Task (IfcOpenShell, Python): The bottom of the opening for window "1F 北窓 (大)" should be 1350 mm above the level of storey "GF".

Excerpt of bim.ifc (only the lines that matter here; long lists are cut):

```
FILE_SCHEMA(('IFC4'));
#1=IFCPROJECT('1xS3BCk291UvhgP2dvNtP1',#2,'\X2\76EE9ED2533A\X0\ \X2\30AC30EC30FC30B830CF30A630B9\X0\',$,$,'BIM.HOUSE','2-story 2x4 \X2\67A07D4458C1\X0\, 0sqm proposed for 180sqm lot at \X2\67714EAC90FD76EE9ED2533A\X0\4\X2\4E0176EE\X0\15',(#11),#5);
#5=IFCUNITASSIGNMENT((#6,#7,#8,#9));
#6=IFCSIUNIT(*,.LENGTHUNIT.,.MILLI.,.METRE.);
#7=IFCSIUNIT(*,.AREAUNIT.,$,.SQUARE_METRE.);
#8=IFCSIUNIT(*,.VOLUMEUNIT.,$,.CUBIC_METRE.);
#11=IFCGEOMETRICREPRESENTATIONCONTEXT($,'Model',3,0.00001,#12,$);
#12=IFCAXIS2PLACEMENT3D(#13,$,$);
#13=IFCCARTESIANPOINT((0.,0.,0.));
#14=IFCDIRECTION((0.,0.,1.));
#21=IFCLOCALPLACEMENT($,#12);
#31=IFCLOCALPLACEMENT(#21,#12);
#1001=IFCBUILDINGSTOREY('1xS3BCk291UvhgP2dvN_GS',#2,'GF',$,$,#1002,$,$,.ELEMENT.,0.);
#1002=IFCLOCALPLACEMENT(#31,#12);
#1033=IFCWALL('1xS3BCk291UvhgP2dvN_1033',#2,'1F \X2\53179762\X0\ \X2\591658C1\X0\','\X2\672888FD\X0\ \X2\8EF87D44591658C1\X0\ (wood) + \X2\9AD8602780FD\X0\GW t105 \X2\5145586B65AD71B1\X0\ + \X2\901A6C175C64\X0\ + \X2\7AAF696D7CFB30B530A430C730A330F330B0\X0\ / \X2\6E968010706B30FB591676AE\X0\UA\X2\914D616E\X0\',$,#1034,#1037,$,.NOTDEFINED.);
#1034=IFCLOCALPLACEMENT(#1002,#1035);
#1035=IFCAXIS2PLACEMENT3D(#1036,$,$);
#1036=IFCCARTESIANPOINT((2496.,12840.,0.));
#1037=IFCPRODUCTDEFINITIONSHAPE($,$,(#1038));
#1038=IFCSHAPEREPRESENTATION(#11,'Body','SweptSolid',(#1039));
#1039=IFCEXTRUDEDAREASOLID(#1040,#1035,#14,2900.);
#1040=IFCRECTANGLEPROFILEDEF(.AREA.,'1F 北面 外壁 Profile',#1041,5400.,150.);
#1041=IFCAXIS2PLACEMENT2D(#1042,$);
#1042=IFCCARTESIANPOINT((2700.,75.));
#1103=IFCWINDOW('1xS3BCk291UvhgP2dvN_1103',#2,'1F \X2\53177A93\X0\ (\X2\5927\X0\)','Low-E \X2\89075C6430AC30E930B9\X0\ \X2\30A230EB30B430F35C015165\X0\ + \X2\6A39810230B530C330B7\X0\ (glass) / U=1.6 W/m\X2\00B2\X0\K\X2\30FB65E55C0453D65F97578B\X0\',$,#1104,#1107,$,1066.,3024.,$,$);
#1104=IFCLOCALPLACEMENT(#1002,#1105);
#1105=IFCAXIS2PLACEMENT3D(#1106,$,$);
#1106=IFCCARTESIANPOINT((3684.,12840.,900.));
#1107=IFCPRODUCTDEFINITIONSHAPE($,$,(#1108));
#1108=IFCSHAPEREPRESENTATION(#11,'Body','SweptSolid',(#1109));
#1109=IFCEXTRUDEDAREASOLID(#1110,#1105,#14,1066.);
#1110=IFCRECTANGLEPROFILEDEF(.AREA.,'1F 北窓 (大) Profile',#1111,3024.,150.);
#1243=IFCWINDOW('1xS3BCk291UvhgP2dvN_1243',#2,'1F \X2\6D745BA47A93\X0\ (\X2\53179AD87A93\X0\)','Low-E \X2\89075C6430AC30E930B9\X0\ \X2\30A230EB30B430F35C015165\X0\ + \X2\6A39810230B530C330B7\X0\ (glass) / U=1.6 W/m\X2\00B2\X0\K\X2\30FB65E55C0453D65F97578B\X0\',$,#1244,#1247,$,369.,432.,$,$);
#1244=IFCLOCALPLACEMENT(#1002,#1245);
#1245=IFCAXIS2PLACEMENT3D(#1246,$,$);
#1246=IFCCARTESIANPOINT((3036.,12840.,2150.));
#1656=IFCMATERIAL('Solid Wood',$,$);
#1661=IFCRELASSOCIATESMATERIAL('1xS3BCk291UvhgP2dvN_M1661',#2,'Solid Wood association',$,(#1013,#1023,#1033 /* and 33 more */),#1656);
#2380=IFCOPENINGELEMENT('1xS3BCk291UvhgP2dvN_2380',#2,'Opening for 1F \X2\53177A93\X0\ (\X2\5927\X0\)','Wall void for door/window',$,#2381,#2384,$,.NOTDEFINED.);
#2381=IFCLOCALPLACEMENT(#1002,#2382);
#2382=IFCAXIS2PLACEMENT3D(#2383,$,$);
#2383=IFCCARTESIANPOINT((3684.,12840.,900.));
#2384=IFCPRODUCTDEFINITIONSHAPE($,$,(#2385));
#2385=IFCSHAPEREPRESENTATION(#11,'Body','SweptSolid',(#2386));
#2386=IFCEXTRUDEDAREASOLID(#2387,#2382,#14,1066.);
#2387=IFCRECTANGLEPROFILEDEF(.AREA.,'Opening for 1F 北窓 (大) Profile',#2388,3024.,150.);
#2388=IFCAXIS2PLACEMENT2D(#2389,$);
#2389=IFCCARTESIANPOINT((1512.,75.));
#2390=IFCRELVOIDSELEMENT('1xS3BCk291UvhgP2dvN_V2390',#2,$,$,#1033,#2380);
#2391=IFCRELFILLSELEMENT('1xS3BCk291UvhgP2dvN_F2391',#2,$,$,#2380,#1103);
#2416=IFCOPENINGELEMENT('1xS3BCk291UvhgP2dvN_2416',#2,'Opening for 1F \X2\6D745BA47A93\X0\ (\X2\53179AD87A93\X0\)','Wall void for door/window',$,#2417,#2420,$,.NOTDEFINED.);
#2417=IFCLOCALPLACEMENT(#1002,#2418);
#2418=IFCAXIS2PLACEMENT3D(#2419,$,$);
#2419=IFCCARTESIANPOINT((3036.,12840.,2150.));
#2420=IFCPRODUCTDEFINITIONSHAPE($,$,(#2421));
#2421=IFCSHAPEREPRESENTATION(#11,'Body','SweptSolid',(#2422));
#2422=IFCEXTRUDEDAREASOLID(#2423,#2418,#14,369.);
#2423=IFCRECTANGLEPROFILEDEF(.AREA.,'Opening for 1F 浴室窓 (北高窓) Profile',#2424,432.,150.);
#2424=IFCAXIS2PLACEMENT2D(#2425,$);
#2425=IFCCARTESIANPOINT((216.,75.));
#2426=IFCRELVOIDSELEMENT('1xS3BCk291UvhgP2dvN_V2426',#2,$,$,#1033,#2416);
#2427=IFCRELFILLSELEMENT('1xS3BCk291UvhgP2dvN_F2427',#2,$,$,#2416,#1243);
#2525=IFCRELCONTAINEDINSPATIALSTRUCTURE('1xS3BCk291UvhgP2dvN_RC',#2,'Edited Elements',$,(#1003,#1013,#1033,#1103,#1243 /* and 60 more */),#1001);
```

```python
import numpy as np
import ifcopenshell
import ifcopenshell.api.geometry
import ifcopenshell.geom
import ifcopenshell.util.element
import ifcopenshell.util.placement
import ifcopenshell.util.shape
import ifcopenshell.util.unit

model = ifcopenshell.open("bim.ifc")
unit_scale = ifcopenshell.util.unit.calculate_unit_scale(model)

window = model.by_guid("1xS3BCk291UvhgP2dvN_1103")
opening = window.FillsVoids[0].RelatingOpeningElement
storey = ifcopenshell.util.element.get_container(window, ifc_class="IfcBuildingStorey")
level = ifcopenshell.util.placement.get_local_placement(storey.ObjectPlacement)[2, 3]

# The opening's origin need not be at the sill, so measure its lowest point.
shape = ifcopenshell.geom.create_shape(ifcopenshell.geom.settings(), opening)
bottom = ifcopenshell.util.shape.get_shape_bottom_elevation(shape, shape.geometry) / unit_scale
dz = level + 1350.0 - bottom

shift = np.array([0.0, 0.0, dz])
# The window is not placed relative to its opening, so move both.
for product in (opening, window):
    matrix = ifcopenshell.util.placement.get_local_placement(product.ObjectPlacement)
    matrix[:3, 3] += shift
    ifcopenshell.api.geometry.edit_object_placement(model, product=product, matrix=matrix, is_si=False)

print(f"moved by {dz * unit_scale:+.3f} m")

model.write("bim_rev.ifc")
```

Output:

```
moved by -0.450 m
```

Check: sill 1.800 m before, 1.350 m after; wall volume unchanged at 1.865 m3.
